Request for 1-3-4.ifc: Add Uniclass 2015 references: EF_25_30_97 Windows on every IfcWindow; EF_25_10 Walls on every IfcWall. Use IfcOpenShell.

First a look at what the model holds.

```python
import ifcopenshell

model = ifcopenshell.open("1-3-4.ifc")
print(model.schema)
print("classifications:", [c.Name for c in model.by_type("IfcClassification")])
for ifc_class in ("IfcDoor", "IfcRoof", "IfcStair", "IfcWall", "IfcWindow"):
    print(ifc_class, len(model.by_type(ifc_class)))
```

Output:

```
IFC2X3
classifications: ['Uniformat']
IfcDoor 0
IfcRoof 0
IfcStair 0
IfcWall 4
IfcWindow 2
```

```python
import ifcopenshell
import ifcopenshell.api.classification

model = ifcopenshell.open("1-3-4.ifc")

# IFC2X3 requires Source and Edition and has no link from the project to the system.
system = model.create_entity("IfcClassification", Source="NBS", Edition="2015", Name="Uniclass 2015")

codes = {
    "IfcWindow": ("EF_25_30_97", "Windows"),
    "IfcWall": ("EF_25_10", "Walls"),
}
for ifc_class, (code, name) in codes.items():
    products = model.by_type(ifc_class)
    ifcopenshell.api.classification.add_reference(
        model, products=products, classification=system, identification=code, name=name
    )
    print(code, len(products))

model.write("1-3-4_edited.ifc")
```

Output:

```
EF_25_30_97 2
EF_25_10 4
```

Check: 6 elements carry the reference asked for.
